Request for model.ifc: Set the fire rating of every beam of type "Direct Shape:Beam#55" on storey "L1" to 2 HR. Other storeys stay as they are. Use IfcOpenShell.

First a look at what the model holds.

```python
import ifcopenshell
import ifcopenshell.util.element

model = ifcopenshell.open("model.ifc")
print(model.schema)
storey = next(s for s in model.by_type("IfcBuildingStorey") if s.Name == "L1")
beams = [e for e in ifcopenshell.util.element.get_decomposition(storey) if e.is_a("IfcBeam")]
seen = {}
for e in beams:
    element_type = ifcopenshell.util.element.get_type(e)
    key = (element_type.Name if element_type != e and element_type else None, ifcopenshell.util.element.get_pset(e, "Pset_BeamCommon", "FireRating"))
    seen[key] = seen.get(key, 0) + 1
for (name, value), count in sorted(seen.items(), key=str):
    print(count, "x", name, "|", value)
```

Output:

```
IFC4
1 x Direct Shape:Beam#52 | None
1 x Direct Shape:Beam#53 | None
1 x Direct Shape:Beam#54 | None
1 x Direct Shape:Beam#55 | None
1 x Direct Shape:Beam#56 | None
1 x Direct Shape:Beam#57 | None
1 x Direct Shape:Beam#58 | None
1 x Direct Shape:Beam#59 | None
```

```python
import ifcopenshell
import ifcopenshell.api.pset
import ifcopenshell.util.element

model = ifcopenshell.open("model.ifc")

storey = next(s for s in model.by_type("IfcBuildingStorey") if s.Name == "L1")
beams = [e for e in ifcopenshell.util.element.get_decomposition(storey) if e.is_a("IfcBeam")]

count = 0
for e in beams:
    element_type = ifcopenshell.util.element.get_type(e)
    if element_type in (None, e) or element_type.Name != "Direct Shape:Beam#55":
        continue
    # add_pset returns the element's existing set when there is one.
    pset = ifcopenshell.api.pset.add_pset(model, product=e, name="Pset_BeamCommon")
    ifcopenshell.api.pset.edit_pset(model, pset=pset, properties={"FireRating": "2 HR"})
    count += 1

print(count, "beams updated")

model.write("model_rev.ifc")
```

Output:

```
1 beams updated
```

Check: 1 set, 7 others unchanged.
